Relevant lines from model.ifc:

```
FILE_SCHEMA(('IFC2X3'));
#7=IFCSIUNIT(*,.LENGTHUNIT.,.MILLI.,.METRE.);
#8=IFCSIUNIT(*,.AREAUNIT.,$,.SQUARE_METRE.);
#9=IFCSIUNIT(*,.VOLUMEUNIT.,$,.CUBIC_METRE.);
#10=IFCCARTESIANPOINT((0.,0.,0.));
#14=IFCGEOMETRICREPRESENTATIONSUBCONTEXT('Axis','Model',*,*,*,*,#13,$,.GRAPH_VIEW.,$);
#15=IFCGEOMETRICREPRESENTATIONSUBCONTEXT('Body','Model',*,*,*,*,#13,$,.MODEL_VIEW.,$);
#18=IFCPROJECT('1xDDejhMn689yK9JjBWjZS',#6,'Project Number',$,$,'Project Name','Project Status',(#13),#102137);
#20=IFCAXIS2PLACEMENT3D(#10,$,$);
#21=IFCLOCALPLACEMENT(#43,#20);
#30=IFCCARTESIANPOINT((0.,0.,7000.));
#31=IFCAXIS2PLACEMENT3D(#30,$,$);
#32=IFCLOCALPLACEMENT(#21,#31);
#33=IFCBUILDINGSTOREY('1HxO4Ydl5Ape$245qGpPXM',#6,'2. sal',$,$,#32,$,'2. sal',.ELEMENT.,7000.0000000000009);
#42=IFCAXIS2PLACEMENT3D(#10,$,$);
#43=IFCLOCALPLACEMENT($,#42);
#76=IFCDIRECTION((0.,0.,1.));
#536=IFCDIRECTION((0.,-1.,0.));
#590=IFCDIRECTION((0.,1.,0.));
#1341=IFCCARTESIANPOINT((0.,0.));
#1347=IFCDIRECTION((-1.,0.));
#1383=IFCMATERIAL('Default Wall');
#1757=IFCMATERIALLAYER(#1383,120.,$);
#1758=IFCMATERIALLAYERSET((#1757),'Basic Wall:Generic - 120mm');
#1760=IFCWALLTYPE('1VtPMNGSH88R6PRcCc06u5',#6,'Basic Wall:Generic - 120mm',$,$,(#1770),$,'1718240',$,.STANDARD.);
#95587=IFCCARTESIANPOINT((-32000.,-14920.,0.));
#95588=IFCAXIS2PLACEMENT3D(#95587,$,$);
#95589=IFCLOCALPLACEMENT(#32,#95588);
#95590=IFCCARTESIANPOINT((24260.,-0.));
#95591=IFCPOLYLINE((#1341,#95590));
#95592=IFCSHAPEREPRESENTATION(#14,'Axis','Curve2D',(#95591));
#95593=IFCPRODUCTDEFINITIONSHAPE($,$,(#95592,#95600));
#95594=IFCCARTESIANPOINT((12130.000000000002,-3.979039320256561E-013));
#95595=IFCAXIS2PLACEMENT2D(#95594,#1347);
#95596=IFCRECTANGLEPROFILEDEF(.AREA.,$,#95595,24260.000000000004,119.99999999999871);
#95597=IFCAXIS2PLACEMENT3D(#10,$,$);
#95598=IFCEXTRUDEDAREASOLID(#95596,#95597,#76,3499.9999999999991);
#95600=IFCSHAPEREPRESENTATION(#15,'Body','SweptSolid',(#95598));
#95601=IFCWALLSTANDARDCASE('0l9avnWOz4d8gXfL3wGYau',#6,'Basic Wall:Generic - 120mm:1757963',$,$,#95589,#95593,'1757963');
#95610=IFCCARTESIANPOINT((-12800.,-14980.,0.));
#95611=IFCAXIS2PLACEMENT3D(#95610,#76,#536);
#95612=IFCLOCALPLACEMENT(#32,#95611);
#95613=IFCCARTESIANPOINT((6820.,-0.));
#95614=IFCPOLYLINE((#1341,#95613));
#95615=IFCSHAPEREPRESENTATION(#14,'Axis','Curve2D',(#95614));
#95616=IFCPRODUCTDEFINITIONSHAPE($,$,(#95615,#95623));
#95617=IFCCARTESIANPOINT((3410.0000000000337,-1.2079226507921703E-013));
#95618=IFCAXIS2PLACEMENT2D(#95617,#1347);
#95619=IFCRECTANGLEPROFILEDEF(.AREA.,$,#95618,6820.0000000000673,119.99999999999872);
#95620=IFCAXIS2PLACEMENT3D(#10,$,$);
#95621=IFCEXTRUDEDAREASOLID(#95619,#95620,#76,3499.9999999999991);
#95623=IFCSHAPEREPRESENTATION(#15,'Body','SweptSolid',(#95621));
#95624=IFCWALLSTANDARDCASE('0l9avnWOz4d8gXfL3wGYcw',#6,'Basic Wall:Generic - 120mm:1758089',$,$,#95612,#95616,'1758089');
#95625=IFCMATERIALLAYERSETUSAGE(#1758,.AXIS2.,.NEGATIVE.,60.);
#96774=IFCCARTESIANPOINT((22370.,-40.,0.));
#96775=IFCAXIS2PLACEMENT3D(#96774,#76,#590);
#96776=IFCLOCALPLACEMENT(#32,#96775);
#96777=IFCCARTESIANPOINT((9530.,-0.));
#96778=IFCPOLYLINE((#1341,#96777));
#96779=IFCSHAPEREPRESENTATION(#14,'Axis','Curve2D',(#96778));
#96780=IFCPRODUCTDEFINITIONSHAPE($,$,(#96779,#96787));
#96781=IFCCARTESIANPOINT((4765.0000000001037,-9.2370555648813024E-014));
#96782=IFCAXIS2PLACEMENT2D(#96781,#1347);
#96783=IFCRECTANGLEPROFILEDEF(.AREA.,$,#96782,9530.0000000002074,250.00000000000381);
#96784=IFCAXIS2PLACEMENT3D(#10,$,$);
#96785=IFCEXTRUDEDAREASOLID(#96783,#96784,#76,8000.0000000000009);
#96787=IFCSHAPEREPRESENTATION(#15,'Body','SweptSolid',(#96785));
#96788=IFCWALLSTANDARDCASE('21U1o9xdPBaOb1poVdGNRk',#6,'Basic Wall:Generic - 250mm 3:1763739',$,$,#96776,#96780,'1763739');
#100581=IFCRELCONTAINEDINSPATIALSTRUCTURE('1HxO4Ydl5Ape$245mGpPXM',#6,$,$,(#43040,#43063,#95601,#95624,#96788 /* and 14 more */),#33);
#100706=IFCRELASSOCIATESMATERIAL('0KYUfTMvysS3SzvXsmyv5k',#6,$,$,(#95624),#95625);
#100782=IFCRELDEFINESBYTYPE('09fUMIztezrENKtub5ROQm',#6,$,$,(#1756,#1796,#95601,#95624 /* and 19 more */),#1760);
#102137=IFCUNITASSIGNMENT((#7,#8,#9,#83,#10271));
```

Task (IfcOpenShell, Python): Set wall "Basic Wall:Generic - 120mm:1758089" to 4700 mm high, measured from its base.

```python
import ifcopenshell
import ifcopenshell.geom
import ifcopenshell.util.representation
import ifcopenshell.util.shape
import ifcopenshell.util.unit

model = ifcopenshell.open("model.ifc")
unit_scale = ifcopenshell.util.unit.calculate_unit_scale(model)
settings = ifcopenshell.geom.settings()


def volume(element):
    """Net volume in cubic metres, openings subtracted."""
    shape = ifcopenshell.geom.create_shape(settings, element)
    return ifcopenshell.util.shape.get_volume(shape.geometry)


wall = model.by_guid("0l9avnWOz4d8gXfL3wGYcw")
before = volume(wall)

body = ifcopenshell.util.representation.get_representation(wall, "Model", "Body")
solid = body.Items[0]
old_height = solid.Depth
solid.Depth = 4.7 / unit_scale
after = volume(wall)

print(f"height {old_height:g} -> {solid.Depth:g}, volume {before:.3f} -> {after:.3f} m3")

model.write("model_updated.ifc")
```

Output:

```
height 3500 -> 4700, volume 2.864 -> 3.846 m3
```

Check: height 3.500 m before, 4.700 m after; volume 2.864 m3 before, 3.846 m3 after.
